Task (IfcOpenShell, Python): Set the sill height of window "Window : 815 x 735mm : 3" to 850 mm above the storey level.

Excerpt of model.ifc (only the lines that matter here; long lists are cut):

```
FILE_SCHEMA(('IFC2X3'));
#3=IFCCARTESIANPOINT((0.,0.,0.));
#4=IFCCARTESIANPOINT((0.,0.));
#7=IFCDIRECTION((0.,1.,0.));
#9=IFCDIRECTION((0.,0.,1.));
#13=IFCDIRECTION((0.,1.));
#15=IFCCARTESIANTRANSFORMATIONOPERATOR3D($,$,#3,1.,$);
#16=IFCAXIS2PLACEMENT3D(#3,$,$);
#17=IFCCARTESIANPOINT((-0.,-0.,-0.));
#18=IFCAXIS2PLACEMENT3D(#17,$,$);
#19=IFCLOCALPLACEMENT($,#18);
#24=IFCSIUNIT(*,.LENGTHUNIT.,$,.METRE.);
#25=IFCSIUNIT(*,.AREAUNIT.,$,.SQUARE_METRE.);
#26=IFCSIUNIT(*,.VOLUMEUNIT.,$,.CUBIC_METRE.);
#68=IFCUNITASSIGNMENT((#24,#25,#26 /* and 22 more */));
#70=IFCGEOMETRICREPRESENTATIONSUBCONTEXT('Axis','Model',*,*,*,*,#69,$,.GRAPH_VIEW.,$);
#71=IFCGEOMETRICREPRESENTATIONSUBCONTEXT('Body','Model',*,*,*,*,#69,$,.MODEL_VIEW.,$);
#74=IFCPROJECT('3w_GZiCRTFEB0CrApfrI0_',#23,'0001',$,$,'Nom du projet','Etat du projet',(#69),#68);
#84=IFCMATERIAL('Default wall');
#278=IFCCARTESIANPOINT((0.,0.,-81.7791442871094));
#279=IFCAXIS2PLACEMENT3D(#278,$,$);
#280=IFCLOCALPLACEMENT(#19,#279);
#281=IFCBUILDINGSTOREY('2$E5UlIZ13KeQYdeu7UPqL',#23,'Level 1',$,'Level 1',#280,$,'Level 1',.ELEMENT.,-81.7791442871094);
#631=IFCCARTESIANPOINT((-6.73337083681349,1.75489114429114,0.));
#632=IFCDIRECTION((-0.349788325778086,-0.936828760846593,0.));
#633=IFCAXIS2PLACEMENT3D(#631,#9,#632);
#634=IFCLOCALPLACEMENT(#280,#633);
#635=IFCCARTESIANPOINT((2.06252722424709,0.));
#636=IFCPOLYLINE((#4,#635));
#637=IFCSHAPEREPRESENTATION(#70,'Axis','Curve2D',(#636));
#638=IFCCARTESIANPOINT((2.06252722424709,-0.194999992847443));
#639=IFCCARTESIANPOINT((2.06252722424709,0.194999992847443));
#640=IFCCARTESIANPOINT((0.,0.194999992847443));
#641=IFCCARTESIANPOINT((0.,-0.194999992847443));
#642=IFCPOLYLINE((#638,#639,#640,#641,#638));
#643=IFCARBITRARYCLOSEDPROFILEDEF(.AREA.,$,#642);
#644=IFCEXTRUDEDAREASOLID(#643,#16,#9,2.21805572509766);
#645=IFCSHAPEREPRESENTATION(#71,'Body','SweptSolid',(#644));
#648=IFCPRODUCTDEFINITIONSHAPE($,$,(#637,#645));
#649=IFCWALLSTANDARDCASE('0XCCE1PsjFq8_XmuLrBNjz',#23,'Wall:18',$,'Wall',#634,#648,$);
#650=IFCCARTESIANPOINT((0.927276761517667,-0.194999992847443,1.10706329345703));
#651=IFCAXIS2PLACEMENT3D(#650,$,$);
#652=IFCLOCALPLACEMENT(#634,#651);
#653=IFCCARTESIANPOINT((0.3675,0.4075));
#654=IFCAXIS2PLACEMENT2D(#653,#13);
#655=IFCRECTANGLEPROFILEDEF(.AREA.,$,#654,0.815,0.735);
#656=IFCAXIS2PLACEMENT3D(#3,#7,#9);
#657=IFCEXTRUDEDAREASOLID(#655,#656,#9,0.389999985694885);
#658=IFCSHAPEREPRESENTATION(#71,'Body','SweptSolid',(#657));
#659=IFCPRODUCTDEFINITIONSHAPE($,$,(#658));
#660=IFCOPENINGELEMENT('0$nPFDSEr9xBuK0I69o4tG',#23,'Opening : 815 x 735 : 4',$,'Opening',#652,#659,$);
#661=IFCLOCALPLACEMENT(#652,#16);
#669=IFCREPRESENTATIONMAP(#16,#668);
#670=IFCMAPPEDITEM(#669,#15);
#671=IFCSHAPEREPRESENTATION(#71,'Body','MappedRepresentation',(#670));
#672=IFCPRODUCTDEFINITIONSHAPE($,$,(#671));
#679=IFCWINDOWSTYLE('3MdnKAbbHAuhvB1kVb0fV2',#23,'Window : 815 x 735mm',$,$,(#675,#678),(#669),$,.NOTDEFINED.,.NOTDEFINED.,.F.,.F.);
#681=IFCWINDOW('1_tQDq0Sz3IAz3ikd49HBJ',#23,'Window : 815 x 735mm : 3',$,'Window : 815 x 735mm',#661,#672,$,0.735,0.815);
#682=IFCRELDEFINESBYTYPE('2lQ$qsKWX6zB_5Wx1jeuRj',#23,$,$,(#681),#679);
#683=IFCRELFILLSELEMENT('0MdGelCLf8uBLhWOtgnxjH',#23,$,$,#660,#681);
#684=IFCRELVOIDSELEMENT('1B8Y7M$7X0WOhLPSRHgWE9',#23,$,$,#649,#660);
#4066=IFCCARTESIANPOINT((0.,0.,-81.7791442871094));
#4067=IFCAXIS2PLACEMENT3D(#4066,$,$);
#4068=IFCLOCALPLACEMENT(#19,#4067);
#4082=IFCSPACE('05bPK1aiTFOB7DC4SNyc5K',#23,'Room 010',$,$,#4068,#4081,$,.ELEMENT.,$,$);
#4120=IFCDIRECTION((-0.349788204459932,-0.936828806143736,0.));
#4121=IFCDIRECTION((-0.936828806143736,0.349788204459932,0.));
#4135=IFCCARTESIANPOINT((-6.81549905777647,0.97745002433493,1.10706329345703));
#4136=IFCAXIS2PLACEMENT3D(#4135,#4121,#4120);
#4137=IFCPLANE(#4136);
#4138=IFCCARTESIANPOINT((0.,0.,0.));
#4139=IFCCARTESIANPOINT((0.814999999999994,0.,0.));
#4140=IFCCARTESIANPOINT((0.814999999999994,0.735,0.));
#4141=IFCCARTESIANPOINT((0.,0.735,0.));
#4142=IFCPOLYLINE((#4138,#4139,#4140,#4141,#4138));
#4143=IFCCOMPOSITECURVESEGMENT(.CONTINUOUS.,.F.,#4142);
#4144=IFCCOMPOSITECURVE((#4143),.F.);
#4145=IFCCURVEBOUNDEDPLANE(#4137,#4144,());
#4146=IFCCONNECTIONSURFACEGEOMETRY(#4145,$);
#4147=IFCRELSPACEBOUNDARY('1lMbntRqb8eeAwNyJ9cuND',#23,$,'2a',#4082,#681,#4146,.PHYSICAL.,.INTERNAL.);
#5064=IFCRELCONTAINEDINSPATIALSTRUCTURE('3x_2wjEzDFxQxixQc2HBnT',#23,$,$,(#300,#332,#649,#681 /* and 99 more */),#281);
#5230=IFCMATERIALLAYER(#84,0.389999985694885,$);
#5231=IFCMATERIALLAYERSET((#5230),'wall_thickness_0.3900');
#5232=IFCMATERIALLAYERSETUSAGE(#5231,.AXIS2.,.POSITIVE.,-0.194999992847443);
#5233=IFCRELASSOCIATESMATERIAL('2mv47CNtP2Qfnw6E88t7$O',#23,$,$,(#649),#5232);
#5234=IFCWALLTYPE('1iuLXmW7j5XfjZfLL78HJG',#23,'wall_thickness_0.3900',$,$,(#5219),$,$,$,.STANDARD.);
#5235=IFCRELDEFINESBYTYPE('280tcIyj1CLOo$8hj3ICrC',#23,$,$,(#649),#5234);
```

```python
import numpy as np
import ifcopenshell
import ifcopenshell.api.geometry
import ifcopenshell.geom
import ifcopenshell.util.element
import ifcopenshell.util.placement
import ifcopenshell.util.shape
import ifcopenshell.util.unit

model = ifcopenshell.open("model.ifc")
unit_scale = ifcopenshell.util.unit.calculate_unit_scale(model)

window = model.by_guid("1_tQDq0Sz3IAz3ikd49HBJ")
opening = window.FillsVoids[0].RelatingOpeningElement
storey = ifcopenshell.util.element.get_container(window, ifc_class="IfcBuildingStorey")
level = ifcopenshell.util.placement.get_local_placement(storey.ObjectPlacement)[2, 3]

# The opening's origin need not be at the sill, so measure its lowest point.
shape = ifcopenshell.geom.create_shape(ifcopenshell.geom.settings(), opening)
bottom = ifcopenshell.util.shape.get_shape_bottom_elevation(shape, shape.geometry) / unit_scale
dz = level + 0.85 / unit_scale - bottom

shift = np.array([0.0, 0.0, dz])
# The window is placed relative to its opening, so it follows when the opening moves.
matrix = ifcopenshell.util.placement.get_local_placement(opening.ObjectPlacement)
matrix[:3, 3] += shift
ifcopenshell.api.geometry.edit_object_placement(
    model, product=opening, matrix=matrix, is_si=False, should_transform_children=True
)

# Space boundary surfaces are stored in each space's coordinates; move them too.
for rel in window.ProvidesBoundaries:
    if not rel.ConnectionGeometry:
        continue
    surface = rel.ConnectionGeometry.SurfaceOnRelatingElement.BasisSurface
    space_matrix = ifcopenshell.util.placement.get_local_placement(rel.RelatingSpace.ObjectPlacement)
    point = np.array(surface.Position.Location.Coordinates) + space_matrix[:3, :3].T @ shift
    surface.Position = model.createIfcAxis2Placement3D(
        model.createIfcCartesianPoint(point.tolist()), surface.Position.Axis, surface.Position.RefDirection
    )

print(f"moved by {dz * unit_scale:+.3f} m")

model.write("model_rev.ifc")
```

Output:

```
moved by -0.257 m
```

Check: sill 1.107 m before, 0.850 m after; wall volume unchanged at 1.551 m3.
